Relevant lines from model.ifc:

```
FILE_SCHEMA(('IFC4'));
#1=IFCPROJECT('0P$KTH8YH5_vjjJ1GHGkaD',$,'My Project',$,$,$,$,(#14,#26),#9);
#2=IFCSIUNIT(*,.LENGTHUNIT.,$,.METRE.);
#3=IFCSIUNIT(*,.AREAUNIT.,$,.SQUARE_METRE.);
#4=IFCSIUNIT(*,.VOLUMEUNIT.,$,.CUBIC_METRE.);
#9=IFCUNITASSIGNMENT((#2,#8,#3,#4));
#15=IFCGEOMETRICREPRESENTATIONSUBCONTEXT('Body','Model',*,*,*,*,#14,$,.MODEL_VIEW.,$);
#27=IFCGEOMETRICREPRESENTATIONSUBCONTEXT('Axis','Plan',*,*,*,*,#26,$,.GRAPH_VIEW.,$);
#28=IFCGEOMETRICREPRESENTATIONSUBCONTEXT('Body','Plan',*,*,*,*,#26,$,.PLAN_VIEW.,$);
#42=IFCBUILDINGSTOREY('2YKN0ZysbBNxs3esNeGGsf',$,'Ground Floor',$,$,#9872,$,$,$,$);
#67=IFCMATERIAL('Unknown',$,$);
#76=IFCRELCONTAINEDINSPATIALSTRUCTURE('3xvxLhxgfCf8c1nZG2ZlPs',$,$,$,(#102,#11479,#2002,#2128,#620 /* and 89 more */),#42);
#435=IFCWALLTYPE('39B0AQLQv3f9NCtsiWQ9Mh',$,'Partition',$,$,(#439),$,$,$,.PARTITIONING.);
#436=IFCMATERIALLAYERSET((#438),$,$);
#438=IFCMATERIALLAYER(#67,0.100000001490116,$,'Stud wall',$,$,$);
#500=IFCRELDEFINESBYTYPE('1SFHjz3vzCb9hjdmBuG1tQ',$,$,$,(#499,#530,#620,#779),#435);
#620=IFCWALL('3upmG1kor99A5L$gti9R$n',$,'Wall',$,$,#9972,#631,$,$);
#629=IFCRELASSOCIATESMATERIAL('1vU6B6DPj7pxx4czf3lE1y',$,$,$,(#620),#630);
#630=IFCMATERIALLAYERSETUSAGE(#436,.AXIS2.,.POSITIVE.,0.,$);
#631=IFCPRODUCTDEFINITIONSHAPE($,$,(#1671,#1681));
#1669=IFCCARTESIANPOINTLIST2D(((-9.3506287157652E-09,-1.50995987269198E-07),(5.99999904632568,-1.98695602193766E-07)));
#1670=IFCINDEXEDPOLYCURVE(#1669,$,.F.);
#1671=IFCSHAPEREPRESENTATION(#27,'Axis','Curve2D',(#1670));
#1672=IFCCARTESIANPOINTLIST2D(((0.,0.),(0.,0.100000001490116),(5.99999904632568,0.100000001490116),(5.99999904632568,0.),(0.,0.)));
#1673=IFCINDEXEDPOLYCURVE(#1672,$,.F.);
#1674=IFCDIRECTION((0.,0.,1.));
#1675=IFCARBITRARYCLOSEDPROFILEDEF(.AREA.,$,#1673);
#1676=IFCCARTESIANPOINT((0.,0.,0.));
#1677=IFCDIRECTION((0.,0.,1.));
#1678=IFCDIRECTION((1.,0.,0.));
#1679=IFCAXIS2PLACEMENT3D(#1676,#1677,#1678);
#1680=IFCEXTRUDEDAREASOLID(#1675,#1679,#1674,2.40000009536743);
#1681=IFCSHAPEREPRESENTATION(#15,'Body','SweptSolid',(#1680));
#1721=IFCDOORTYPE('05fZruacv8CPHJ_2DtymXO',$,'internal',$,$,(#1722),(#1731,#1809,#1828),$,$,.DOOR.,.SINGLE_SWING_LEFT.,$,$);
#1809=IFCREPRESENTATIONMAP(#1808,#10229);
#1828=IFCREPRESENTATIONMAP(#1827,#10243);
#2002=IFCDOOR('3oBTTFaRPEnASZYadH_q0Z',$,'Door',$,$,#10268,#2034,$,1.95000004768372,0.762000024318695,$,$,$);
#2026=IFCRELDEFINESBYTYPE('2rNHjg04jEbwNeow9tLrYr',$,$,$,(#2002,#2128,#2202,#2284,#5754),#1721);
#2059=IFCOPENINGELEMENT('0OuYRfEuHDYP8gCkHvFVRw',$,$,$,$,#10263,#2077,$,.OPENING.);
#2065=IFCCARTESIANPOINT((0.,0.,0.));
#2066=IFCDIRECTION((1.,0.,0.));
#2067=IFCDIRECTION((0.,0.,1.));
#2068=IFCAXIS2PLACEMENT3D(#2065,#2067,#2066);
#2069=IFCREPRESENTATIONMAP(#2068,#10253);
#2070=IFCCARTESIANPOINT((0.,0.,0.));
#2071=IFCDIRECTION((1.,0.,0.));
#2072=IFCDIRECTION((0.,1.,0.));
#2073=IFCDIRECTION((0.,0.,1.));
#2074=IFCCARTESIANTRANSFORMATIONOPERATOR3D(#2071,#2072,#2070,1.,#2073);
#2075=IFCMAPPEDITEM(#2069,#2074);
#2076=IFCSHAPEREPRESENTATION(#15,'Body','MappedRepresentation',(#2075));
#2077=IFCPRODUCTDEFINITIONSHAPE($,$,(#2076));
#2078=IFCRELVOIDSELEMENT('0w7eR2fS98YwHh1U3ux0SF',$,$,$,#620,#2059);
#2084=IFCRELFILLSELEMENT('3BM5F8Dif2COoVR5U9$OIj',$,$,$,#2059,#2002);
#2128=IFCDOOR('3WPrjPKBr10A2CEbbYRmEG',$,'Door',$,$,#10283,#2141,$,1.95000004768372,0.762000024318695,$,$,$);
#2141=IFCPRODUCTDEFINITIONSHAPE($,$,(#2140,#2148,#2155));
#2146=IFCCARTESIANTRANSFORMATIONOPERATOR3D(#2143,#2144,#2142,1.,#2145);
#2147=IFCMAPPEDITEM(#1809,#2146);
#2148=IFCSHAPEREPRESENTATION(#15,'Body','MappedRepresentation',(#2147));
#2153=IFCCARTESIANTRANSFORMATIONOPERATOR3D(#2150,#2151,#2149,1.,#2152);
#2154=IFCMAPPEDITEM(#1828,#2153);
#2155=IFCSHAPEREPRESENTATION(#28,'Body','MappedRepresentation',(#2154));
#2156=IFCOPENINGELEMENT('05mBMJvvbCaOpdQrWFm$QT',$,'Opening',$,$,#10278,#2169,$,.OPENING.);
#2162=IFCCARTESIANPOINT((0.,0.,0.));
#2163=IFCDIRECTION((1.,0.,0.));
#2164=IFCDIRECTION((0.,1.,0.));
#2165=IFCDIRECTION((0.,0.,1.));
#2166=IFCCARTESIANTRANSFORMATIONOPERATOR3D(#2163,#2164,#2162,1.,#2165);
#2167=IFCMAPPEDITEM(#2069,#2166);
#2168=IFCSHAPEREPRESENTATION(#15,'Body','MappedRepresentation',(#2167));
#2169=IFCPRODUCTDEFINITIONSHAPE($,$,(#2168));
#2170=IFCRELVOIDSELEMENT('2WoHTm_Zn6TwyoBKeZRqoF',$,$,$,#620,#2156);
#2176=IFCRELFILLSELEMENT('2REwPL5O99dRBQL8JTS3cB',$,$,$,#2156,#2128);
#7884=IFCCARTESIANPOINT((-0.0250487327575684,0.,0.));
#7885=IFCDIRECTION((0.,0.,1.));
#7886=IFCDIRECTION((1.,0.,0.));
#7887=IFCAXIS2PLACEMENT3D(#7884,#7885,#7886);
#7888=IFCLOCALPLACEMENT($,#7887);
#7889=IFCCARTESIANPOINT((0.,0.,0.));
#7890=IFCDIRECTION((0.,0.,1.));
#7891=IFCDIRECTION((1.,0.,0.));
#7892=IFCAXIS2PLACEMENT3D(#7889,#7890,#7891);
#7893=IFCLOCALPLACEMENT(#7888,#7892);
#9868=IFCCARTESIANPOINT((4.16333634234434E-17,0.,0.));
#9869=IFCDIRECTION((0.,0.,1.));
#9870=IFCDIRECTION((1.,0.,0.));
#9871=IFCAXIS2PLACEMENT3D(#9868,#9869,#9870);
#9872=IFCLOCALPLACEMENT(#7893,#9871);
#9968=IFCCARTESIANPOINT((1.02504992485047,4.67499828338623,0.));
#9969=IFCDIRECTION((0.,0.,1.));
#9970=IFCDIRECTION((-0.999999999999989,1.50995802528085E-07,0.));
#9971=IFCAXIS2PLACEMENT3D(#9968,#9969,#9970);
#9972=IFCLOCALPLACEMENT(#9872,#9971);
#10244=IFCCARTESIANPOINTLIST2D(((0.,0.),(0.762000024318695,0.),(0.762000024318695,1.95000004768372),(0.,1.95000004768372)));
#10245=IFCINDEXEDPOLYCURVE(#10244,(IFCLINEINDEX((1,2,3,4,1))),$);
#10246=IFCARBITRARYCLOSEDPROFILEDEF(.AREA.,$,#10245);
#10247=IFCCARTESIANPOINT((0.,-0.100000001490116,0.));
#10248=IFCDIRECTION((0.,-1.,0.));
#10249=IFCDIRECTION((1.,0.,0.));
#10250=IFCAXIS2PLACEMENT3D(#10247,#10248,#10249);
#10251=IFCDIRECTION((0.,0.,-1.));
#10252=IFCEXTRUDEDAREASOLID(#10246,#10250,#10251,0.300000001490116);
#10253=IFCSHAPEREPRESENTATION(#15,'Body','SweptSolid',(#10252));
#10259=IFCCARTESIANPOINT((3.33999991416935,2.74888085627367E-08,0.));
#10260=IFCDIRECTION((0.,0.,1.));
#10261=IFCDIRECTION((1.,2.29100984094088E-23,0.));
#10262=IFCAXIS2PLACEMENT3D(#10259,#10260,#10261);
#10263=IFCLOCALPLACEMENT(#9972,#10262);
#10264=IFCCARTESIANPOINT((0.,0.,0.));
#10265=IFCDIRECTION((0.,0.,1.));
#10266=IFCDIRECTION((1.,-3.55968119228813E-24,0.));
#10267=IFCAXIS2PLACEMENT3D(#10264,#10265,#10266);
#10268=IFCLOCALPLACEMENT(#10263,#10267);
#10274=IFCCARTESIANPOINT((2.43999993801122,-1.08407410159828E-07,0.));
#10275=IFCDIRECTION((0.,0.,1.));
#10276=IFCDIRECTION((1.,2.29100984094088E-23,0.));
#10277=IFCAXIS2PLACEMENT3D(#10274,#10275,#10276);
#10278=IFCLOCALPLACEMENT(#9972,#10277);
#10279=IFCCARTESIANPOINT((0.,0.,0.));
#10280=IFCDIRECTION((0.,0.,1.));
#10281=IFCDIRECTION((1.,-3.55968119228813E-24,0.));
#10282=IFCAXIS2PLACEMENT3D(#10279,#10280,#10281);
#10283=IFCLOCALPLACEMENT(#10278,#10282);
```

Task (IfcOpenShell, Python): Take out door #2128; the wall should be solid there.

```python
import ifcopenshell
import ifcopenshell.api.feature
import ifcopenshell.api.root
import ifcopenshell.geom
import ifcopenshell.util.shape

model = ifcopenshell.open("model.ifc")
settings = ifcopenshell.geom.settings()


def volume(element):
    """Net volume in cubic metres, openings subtracted."""
    shape = ifcopenshell.geom.create_shape(settings, element)
    return ifcopenshell.util.shape.get_volume(shape.geometry)


door = model.by_guid("3WPrjPKBr10A2CEbbYRmEG")
opening = door.FillsVoids[0].RelatingOpeningElement
wall = opening.VoidsElements[0].RelatingBuildingElement
before = volume(wall)

ifcopenshell.api.root.remove_product(model, product=door)
ifcopenshell.api.feature.remove_feature(model, feature=opening)

after = volume(wall)

print(f"wall volume {before:.3f} -> {after:.3f} m3")

model.write("model_v2.ifc")
```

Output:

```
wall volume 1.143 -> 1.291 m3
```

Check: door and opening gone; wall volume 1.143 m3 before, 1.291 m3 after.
